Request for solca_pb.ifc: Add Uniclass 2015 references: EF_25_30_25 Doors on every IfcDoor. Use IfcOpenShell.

First a look at what the model holds.

```python
import ifcopenshell

model = ifcopenshell.open("solca_pb.ifc")
print(model.schema)
print("classifications:", [c.Name for c in model.by_type("IfcClassification")])
for ifc_class in ("IfcDoor", "IfcRoof", "IfcStair", "IfcWall", "IfcWindow"):
    print(ifc_class, len(model.by_type(ifc_class)))
```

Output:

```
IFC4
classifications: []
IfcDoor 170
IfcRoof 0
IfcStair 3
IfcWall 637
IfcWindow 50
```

```python
import ifcopenshell
import ifcopenshell.api.classification

model = ifcopenshell.open("solca_pb.ifc")

system = ifcopenshell.api.classification.add_classification(model, classification="Uniclass 2015")

codes = {
    "IfcDoor": ("EF_25_30_25", "Doors"),
}
for ifc_class, (code, name) in codes.items():
    products = model.by_type(ifc_class)
    ifcopenshell.api.classification.add_reference(
        model, products=products, classification=system, identification=code, name=name
    )
    print(code, len(products))

model.write("solca_pb_updated.ifc")
```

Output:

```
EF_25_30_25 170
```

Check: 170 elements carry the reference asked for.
